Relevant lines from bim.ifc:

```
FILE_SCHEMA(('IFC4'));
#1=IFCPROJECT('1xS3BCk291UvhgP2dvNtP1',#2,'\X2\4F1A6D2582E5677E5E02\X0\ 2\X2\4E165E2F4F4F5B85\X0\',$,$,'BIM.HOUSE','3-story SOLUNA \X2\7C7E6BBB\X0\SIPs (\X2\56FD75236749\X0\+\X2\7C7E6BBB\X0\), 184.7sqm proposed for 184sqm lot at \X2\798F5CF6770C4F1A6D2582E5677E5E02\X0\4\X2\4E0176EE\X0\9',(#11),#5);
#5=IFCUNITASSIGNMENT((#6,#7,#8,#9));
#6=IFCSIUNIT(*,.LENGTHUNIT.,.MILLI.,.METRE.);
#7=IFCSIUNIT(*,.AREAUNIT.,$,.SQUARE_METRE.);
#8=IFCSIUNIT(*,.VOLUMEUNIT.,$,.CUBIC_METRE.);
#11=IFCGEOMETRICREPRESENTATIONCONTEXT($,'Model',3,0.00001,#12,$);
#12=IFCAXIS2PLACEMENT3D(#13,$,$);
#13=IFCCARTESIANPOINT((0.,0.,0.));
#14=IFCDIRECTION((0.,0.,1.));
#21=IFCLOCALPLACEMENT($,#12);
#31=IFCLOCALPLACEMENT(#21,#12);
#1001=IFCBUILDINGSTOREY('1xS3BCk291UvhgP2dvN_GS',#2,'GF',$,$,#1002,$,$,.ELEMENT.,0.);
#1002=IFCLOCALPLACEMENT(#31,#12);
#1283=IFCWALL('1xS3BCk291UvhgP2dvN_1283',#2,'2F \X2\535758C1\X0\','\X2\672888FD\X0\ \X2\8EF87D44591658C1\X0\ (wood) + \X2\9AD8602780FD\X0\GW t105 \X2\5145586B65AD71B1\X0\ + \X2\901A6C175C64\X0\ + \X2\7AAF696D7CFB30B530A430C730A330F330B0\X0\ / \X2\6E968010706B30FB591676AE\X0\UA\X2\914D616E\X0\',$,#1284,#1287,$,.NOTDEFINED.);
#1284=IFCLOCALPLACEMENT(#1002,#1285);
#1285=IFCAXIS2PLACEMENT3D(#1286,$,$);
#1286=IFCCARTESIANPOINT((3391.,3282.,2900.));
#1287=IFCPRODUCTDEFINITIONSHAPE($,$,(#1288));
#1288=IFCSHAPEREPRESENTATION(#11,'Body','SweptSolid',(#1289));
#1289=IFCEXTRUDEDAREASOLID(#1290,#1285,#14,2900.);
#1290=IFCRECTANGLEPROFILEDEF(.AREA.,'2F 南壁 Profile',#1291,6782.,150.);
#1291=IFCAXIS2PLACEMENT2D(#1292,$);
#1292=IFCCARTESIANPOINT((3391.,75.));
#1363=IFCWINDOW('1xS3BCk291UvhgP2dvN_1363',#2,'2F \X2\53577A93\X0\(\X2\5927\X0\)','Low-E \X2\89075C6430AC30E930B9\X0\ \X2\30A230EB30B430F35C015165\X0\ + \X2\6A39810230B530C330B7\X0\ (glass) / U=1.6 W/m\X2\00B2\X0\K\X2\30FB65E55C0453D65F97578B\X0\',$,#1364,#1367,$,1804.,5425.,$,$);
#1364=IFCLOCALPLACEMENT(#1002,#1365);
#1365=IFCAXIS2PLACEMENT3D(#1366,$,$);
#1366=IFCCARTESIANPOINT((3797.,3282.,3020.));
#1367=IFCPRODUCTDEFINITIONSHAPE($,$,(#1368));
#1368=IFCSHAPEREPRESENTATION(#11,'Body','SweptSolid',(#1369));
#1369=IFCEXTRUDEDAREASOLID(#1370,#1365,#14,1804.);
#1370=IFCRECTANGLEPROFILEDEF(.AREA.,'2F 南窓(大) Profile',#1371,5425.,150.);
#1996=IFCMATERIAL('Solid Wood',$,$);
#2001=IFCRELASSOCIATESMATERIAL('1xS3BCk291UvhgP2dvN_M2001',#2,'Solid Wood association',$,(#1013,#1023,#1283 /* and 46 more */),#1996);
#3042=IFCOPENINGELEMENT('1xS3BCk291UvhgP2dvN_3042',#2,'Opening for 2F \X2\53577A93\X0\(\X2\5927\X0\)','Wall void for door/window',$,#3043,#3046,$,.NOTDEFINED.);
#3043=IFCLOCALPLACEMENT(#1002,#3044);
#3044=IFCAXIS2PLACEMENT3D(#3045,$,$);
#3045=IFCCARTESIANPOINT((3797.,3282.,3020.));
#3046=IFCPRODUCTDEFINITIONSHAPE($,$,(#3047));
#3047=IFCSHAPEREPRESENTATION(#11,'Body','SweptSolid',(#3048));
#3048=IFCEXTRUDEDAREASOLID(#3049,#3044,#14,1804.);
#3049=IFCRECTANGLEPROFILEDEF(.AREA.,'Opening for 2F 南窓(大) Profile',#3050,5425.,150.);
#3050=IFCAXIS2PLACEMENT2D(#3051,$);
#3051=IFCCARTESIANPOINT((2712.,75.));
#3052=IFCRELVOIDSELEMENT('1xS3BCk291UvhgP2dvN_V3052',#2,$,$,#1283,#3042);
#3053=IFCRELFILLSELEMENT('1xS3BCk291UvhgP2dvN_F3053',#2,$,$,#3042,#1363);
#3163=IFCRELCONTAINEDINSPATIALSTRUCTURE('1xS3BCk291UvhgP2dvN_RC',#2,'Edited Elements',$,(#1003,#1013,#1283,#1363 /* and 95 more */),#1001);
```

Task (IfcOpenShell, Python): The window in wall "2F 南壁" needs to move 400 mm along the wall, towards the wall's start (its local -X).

```python
import ifcopenshell
import ifcopenshell.api.geometry
import ifcopenshell.util.placement

model = ifcopenshell.open("bim.ifc")

window = model.by_guid("1xS3BCk291UvhgP2dvN_1363")
opening = window.FillsVoids[0].RelatingOpeningElement
wall = opening.VoidsElements[0].RelatingBuildingElement

wall_matrix = ifcopenshell.util.placement.get_local_placement(wall.ObjectPlacement)
shift = wall_matrix[:3, 0] * -400.0
before = ifcopenshell.util.placement.get_local_placement(window.ObjectPlacement)[:3, 3].copy()

# The window is not placed relative to its opening, so move both.
for product in (opening, window):
    matrix = ifcopenshell.util.placement.get_local_placement(product.ObjectPlacement)
    matrix[:3, 3] += shift
    ifcopenshell.api.geometry.edit_object_placement(model, product=product, matrix=matrix, is_si=False)

after = ifcopenshell.util.placement.get_local_placement(window.ObjectPlacement)[:3, 3]
print("window moved by", (after - before).round(3) + 0.0)

model.write("bim_updated.ifc")
```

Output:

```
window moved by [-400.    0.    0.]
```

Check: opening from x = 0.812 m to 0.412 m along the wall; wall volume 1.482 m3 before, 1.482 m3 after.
